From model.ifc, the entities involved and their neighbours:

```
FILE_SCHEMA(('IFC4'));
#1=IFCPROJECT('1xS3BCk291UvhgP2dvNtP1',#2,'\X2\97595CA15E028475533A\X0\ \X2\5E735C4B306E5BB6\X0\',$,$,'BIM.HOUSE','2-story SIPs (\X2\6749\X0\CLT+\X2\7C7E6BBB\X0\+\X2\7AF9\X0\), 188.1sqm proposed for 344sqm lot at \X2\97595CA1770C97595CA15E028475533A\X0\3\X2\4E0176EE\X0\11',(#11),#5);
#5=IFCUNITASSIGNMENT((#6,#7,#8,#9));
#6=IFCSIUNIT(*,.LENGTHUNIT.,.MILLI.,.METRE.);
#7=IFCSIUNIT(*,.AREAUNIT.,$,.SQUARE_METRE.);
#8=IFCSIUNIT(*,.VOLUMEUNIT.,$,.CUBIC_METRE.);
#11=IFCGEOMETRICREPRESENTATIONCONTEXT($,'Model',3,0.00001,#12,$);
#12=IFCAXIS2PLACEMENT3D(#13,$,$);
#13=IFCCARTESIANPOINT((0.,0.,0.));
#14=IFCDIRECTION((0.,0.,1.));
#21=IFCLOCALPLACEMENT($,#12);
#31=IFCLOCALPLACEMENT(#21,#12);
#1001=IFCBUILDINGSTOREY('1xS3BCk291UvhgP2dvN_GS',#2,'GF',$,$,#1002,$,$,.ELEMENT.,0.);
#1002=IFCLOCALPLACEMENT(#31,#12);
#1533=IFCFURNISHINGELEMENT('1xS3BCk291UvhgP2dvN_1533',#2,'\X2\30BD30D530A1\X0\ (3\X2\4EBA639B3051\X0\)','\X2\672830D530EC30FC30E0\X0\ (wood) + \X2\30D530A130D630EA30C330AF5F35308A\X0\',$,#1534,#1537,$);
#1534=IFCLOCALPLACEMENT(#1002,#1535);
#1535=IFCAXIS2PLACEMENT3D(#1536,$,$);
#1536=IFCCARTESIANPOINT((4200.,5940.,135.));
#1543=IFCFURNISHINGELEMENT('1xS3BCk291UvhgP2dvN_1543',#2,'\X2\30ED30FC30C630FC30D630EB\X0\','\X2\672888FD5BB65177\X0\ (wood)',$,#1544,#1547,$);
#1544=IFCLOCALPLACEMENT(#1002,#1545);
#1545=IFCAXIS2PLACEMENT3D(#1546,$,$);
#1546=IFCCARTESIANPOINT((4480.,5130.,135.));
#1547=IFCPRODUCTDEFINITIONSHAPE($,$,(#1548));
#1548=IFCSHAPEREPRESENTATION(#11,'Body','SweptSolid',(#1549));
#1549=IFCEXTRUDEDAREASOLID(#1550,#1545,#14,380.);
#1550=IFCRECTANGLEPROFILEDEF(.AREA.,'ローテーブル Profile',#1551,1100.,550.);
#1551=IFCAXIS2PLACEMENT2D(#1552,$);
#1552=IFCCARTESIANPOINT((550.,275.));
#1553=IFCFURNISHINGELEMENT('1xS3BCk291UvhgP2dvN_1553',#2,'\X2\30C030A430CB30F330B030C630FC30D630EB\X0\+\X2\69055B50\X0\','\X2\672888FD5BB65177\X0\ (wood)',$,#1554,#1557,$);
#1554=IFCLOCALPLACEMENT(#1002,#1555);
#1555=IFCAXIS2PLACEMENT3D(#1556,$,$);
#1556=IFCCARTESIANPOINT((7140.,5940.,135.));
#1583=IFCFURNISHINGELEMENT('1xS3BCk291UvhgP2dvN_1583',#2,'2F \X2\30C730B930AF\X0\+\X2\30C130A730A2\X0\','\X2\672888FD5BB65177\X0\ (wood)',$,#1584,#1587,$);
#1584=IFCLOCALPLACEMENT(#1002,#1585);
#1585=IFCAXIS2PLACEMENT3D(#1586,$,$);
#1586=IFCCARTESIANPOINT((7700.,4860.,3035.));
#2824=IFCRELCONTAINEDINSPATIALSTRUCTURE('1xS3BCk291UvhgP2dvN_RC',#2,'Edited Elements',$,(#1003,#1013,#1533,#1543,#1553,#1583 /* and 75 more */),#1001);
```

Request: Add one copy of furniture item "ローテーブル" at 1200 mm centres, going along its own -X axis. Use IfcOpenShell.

```python
import ifcopenshell
import ifcopenshell.api.geometry
import ifcopenshell.api.root
import ifcopenshell.util.element
import ifcopenshell.util.placement
import ifcopenshell.util.unit

model = ifcopenshell.open("model.ifc")
unit_scale = ifcopenshell.util.unit.calculate_unit_scale(model)


def reuse_history(source, copy):
    """copy_class also copies each property set's owner history, people and application; keep the originals."""
    for rel in copy.IsDefinedBy:
        if rel.is_a("IfcRelDefinesByProperties") and (history := rel.RelatingPropertyDefinition.OwnerHistory):
            rel.RelatingPropertyDefinition.OwnerHistory = source.OwnerHistory
            ifcopenshell.util.element.remove_deep2(model, history)


source = model.by_id(1543)
base = ifcopenshell.util.placement.get_local_placement(source.ObjectPlacement)
step = -base[:3, 0] * 1.2 / unit_scale

for i in range(1, 2):
    copy = ifcopenshell.api.root.copy_class(model, product=source)
    copy.Representation = ifcopenshell.util.element.copy_deep(
        model, source.Representation, exclude=["IfcGeometricRepresentationContext", "IfcRepresentationMap"]
    )
    reuse_history(source, copy)
    matrix = base.copy()
    matrix[:3, 3] += i * step
    print("added at", matrix[:3, 3].round(3) + 0.0)
    ifcopenshell.api.geometry.edit_object_placement(model, product=copy, matrix=matrix, is_si=False)

model.write("model_v2.ifc")
```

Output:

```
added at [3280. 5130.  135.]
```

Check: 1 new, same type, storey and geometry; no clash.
